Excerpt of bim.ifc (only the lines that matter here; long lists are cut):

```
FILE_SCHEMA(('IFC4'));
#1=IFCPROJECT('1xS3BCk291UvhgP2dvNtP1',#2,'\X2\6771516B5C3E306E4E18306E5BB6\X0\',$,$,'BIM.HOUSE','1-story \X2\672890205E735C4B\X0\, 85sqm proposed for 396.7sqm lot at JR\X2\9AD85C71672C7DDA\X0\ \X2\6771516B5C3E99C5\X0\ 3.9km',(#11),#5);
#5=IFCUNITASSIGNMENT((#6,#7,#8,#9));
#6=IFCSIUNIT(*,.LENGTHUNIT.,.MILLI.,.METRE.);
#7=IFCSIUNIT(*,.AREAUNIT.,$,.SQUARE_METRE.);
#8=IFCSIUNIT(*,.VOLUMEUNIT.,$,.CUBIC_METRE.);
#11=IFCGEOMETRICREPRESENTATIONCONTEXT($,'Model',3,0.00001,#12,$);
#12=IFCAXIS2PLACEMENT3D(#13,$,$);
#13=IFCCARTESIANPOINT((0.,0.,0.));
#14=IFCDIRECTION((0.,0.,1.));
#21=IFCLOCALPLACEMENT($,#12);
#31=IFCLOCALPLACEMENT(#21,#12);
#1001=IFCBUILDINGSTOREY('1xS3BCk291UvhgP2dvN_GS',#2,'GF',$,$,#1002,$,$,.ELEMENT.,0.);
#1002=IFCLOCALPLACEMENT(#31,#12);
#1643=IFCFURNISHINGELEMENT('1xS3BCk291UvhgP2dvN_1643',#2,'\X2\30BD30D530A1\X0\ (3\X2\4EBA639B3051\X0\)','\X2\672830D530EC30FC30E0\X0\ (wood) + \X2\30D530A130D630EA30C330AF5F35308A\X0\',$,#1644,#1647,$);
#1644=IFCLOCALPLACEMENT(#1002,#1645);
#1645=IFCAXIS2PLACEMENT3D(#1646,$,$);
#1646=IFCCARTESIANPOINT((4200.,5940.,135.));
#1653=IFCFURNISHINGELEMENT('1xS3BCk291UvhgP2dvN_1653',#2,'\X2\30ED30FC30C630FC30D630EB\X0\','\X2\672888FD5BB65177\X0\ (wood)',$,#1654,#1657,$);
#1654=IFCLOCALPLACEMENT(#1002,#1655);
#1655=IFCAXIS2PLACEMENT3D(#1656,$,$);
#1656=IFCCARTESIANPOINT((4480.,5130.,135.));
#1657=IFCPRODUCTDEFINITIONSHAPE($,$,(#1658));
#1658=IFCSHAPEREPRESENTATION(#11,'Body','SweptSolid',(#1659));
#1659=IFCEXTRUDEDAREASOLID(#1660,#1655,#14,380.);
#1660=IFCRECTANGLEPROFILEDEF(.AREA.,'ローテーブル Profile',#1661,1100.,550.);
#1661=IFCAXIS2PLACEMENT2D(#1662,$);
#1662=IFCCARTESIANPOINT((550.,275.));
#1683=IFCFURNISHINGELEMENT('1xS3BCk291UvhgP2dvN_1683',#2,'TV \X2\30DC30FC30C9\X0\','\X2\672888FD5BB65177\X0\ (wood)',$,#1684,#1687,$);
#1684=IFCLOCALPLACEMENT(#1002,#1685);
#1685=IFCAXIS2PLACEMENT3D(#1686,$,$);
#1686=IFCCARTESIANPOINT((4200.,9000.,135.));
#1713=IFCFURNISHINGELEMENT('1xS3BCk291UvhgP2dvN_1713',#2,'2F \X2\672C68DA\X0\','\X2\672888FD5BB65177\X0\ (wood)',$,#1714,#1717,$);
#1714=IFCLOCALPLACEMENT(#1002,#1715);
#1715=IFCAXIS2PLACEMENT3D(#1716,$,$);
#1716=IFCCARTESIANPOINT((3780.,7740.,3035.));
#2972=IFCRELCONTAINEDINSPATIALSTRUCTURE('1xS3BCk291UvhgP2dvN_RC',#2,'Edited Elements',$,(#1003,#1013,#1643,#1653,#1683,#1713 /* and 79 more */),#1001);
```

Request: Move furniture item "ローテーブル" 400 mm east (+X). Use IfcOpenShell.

```python
import ifcopenshell
import ifcopenshell.api.geometry
import ifcopenshell.util.placement
import ifcopenshell.util.unit

model = ifcopenshell.open("bim.ifc")
unit_scale = ifcopenshell.util.unit.calculate_unit_scale(model)

item = model.by_guid("1xS3BCk291UvhgP2dvN_1653")
matrix = ifcopenshell.util.placement.get_local_placement(item.ObjectPlacement)
matrix[0, 3] += 0.4 / unit_scale
ifcopenshell.api.geometry.edit_object_placement(model, product=item, matrix=matrix, is_si=False)

print(ifcopenshell.util.placement.get_local_placement(item.ObjectPlacement).round(3) + 0.0)

model.write("bim-out.ifc")
```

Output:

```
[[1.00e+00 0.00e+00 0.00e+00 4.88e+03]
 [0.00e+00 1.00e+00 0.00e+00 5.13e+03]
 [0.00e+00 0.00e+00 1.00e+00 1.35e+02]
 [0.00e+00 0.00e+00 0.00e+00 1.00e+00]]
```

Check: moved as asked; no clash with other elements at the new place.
